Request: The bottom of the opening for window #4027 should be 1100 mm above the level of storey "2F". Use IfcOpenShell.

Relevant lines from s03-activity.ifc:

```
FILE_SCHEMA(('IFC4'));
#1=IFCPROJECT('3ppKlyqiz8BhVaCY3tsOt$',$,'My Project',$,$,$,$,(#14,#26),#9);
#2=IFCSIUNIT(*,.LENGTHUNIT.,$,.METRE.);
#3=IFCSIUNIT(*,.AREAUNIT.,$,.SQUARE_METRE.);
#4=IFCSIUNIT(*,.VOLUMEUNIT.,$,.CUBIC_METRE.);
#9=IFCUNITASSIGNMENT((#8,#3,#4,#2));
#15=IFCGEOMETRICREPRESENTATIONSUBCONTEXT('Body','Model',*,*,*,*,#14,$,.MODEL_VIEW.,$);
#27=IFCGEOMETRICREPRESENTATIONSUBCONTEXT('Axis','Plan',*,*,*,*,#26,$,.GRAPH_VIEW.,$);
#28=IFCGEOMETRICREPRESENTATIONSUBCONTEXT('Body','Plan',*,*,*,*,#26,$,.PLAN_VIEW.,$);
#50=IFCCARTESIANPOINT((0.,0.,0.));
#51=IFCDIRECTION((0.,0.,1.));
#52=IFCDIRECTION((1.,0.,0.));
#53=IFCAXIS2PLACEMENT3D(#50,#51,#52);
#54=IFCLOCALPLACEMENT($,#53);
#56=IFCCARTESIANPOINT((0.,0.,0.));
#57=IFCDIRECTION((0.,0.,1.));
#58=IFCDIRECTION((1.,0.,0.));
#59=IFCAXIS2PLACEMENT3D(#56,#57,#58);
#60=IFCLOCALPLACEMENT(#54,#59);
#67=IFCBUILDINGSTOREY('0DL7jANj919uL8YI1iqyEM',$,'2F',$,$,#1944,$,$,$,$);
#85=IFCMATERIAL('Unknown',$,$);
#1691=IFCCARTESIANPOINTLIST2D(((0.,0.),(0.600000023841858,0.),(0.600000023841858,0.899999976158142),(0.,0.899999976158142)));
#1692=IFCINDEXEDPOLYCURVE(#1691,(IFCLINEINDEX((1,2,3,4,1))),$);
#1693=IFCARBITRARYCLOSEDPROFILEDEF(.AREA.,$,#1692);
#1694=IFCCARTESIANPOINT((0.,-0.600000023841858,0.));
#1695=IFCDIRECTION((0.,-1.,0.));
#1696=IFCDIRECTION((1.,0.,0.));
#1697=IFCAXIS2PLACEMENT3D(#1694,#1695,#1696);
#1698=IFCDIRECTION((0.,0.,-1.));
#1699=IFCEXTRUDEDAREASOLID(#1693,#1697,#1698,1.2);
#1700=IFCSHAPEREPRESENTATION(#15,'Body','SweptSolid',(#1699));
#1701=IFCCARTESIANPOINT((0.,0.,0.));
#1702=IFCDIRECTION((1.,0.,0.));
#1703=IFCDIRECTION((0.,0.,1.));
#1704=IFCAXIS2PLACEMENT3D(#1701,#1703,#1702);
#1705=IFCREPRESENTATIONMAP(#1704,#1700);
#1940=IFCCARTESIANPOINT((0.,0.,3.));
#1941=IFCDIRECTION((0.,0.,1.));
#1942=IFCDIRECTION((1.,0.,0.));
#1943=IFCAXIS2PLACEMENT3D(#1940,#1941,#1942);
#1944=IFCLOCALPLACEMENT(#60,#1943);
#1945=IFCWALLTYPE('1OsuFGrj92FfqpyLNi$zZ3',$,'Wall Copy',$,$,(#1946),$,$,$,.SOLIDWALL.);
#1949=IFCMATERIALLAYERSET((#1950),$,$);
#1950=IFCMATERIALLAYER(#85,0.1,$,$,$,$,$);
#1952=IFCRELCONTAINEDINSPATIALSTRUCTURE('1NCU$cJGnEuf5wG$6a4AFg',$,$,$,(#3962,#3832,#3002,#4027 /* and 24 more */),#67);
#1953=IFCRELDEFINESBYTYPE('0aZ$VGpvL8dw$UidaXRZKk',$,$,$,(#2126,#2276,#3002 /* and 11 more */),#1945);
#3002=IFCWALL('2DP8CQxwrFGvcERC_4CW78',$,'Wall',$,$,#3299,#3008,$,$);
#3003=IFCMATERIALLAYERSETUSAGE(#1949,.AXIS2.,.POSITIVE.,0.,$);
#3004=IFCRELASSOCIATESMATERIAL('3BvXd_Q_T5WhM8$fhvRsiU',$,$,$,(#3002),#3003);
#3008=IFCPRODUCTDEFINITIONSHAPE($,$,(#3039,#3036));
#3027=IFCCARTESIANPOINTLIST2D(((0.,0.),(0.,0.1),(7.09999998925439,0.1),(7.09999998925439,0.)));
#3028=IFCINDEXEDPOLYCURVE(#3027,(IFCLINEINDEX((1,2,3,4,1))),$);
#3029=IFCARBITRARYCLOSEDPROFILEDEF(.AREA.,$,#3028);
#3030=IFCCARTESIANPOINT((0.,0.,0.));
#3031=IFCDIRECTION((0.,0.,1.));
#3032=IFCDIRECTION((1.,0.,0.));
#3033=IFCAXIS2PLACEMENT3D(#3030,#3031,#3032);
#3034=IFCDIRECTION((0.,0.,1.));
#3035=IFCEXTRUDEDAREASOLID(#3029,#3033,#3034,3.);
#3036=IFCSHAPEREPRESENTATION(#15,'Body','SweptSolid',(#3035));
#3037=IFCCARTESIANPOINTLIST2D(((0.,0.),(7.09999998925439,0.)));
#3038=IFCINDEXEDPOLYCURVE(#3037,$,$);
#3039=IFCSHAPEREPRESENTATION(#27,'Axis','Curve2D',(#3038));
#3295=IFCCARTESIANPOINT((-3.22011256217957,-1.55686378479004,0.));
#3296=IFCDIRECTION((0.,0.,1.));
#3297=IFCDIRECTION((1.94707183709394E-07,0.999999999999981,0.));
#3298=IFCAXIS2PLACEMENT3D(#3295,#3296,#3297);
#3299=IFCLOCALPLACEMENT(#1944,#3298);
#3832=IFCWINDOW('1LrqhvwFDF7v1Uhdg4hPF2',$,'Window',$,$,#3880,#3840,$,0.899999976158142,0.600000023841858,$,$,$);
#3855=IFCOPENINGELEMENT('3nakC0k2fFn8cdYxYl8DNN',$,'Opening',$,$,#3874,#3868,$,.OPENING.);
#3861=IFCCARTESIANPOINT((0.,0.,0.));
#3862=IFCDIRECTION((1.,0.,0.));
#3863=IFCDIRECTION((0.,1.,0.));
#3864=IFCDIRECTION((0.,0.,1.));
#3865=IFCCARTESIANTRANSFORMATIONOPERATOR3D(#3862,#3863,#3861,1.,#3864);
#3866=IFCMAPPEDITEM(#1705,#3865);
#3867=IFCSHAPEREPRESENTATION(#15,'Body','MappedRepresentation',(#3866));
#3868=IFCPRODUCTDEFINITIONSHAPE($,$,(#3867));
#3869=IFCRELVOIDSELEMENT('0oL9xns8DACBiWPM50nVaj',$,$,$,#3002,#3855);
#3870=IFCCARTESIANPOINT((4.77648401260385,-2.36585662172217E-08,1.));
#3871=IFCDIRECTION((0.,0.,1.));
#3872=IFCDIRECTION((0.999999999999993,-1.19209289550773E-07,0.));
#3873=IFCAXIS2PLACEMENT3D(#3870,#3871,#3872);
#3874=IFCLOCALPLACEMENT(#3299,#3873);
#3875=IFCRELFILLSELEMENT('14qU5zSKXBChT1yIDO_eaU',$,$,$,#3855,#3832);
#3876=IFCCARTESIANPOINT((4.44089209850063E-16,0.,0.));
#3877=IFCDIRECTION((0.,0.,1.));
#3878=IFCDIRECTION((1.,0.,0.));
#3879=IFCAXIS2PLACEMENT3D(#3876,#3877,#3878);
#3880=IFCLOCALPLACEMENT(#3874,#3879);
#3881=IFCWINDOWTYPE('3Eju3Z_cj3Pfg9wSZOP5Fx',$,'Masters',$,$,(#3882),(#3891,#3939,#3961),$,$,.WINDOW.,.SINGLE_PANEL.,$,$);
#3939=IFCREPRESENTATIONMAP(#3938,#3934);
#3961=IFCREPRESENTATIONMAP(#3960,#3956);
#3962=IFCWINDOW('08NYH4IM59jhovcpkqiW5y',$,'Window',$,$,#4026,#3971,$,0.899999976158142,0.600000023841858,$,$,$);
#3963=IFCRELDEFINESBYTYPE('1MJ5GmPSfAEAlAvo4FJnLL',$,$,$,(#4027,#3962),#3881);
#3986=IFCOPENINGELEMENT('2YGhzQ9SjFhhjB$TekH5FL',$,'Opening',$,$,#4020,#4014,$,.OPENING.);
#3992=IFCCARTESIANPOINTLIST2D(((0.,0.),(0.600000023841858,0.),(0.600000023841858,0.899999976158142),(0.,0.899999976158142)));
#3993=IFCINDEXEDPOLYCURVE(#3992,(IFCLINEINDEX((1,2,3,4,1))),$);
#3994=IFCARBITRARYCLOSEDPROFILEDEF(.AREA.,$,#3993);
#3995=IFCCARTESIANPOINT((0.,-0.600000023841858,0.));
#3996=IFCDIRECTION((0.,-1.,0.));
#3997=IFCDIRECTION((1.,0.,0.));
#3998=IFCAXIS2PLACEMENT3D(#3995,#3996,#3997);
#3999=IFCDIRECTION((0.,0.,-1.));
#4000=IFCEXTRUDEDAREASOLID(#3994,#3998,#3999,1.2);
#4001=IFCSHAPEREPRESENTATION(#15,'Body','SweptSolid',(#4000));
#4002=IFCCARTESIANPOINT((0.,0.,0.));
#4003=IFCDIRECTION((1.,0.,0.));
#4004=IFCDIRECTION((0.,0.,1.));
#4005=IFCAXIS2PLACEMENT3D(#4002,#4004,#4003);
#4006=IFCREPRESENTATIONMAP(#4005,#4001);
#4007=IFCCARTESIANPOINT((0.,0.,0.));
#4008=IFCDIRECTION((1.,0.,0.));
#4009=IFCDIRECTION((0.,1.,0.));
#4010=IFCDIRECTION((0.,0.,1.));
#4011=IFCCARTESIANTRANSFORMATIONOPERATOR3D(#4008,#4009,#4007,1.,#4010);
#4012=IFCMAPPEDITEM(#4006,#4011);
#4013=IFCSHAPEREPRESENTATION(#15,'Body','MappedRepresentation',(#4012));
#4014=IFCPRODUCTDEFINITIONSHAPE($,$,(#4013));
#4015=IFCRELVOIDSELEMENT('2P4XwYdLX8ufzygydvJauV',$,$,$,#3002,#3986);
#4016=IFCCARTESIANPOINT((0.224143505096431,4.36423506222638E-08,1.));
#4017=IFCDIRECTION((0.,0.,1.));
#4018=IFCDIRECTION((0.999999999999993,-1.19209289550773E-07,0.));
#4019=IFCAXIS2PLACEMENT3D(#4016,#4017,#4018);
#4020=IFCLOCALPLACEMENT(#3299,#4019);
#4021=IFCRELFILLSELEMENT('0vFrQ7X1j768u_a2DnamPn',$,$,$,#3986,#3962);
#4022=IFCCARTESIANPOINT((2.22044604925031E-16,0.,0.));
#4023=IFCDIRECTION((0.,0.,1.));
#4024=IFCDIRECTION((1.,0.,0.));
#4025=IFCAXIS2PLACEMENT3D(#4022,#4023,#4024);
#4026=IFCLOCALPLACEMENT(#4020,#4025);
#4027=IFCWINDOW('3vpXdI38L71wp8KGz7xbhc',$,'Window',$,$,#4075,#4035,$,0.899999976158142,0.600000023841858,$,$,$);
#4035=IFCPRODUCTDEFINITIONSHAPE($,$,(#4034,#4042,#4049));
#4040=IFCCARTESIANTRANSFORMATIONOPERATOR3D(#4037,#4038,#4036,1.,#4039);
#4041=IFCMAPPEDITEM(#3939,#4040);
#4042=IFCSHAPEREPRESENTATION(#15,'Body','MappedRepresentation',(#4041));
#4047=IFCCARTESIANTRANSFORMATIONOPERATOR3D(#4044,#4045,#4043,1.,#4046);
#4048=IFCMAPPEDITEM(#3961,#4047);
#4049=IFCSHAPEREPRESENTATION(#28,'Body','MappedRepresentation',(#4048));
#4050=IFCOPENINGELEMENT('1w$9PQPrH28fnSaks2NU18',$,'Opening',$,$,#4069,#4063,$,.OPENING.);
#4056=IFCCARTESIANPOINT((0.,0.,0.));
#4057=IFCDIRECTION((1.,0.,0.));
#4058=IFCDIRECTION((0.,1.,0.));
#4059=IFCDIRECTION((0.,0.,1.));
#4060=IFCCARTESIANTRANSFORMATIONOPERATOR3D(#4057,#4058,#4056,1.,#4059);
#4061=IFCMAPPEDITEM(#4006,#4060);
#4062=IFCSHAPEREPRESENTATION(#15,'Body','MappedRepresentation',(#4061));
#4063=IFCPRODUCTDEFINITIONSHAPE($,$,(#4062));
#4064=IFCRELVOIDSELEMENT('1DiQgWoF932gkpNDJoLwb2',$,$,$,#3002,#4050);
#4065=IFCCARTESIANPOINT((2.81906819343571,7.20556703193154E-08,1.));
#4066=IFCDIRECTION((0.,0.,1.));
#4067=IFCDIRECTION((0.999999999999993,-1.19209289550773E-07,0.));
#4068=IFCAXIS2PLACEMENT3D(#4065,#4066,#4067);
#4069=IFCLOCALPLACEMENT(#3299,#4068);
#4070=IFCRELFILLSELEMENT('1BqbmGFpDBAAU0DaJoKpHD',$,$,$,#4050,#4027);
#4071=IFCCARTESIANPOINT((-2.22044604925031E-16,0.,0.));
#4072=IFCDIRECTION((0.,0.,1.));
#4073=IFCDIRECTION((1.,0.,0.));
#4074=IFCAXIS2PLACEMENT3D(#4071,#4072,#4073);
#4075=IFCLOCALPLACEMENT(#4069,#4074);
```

```python
import numpy as np
import ifcopenshell
import ifcopenshell.api.geometry
import ifcopenshell.geom
import ifcopenshell.util.element
import ifcopenshell.util.placement
import ifcopenshell.util.shape
import ifcopenshell.util.unit

model = ifcopenshell.open("s03-activity.ifc")
unit_scale = ifcopenshell.util.unit.calculate_unit_scale(model)

window = model.by_id(4027)
opening = window.FillsVoids[0].RelatingOpeningElement
storey = ifcopenshell.util.element.get_container(window, ifc_class="IfcBuildingStorey")
level = ifcopenshell.util.placement.get_local_placement(storey.ObjectPlacement)[2, 3]

# The opening's origin need not be at the sill, so measure its lowest point.
shape = ifcopenshell.geom.create_shape(ifcopenshell.geom.settings(), opening)
bottom = ifcopenshell.util.shape.get_shape_bottom_elevation(shape, shape.geometry) / unit_scale
dz = level + 1.1 / unit_scale - bottom

shift = np.array([0.0, 0.0, dz])
# The window is placed relative to its opening, so it follows when the opening moves.
matrix = ifcopenshell.util.placement.get_local_placement(opening.ObjectPlacement)
matrix[:3, 3] += shift
ifcopenshell.api.geometry.edit_object_placement(
    model, product=opening, matrix=matrix, is_si=False, should_transform_children=True
)

print(f"moved by {dz * unit_scale:+.3f} m")

model.write("s03-activity_rev.ifc")
```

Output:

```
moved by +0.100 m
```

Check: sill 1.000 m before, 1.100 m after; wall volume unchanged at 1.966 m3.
